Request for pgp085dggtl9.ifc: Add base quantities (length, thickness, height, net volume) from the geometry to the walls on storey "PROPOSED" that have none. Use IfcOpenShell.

First a look at what the model holds.

```python
import ifcopenshell
import ifcopenshell.util.element
import ifcopenshell.util.unit

model = ifcopenshell.open("pgp085dggtl9.ifc")
print(model.schema)
for unit_type in ("LENGTHUNIT", "AREAUNIT", "VOLUMEUNIT"):
    print(unit_type, ifcopenshell.util.unit.calculate_unit_scale(model, unit_type))
storey = next(s for s in model.by_type("IfcBuildingStorey") if s.Name == "PROPOSED")
walls = [e for e in ifcopenshell.util.element.get_decomposition(storey) if e.is_a("IfcWall")]
for e in sorted(walls, key=lambda e: e.id()):
    print(e.id(), e.is_a(), e.Name, list(ifcopenshell.util.element.get_psets(e, qtos_only=True)), sep=" | ")
```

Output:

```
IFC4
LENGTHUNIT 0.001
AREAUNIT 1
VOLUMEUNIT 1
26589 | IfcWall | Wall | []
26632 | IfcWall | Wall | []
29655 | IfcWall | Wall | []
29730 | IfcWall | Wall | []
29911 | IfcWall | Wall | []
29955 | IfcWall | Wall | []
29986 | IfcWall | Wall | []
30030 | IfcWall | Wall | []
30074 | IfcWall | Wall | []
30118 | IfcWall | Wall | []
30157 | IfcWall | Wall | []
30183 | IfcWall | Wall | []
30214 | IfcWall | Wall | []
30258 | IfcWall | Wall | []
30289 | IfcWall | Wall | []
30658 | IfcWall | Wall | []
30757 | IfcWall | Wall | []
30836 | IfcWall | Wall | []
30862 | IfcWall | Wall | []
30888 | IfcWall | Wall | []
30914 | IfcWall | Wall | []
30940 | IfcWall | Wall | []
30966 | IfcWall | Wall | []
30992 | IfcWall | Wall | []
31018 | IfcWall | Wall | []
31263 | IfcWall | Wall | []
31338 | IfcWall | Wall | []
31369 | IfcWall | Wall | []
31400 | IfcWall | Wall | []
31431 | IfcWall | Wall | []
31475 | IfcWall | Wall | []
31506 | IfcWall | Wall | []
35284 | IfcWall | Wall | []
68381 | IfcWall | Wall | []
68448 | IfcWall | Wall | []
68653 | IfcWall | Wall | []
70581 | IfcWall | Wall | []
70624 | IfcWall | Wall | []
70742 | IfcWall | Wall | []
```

```python
import ifcopenshell
import ifcopenshell.api.pset
import ifcopenshell.geom
import ifcopenshell.util.element
import ifcopenshell.util.shape
import ifcopenshell.util.unit

model = ifcopenshell.open("pgp085dggtl9.ifc")
unit_scale = ifcopenshell.util.unit.calculate_unit_scale(model)
volume_scale = ifcopenshell.util.unit.calculate_unit_scale(model, "VOLUMEUNIT")
settings = ifcopenshell.geom.settings()

storey = next(s for s in model.by_type("IfcBuildingStorey") if s.Name == "PROPOSED")
walls = [e for e in ifcopenshell.util.element.get_decomposition(storey) if e.is_a("IfcWall")]

for e in sorted(walls, key=lambda e: e.id()):
    if ifcopenshell.util.element.get_psets(e, qtos_only=True, should_inherit=False):
        continue
    # Geometry comes back in metres, in the element's own axes.
    shape = ifcopenshell.geom.create_shape(settings, e)
    values = {
        "Length": ifcopenshell.util.shape.get_x(shape.geometry) / unit_scale,
        "Width": ifcopenshell.util.shape.get_y(shape.geometry) / unit_scale,
        "Height": ifcopenshell.util.shape.get_z(shape.geometry) / unit_scale,
        "NetVolume": ifcopenshell.util.shape.get_volume(shape.geometry) / volume_scale,
    }
    qto = ifcopenshell.api.pset.add_qto(model, product=e, name="Qto_WallBaseQuantities")
    ifcopenshell.api.pset.edit_qto(model, qto=qto, properties=values)
    print(e.id(), {k: round(v, 3) for k, v in values.items()})

model.write("pgp085dggtl9_rev.ifc")
```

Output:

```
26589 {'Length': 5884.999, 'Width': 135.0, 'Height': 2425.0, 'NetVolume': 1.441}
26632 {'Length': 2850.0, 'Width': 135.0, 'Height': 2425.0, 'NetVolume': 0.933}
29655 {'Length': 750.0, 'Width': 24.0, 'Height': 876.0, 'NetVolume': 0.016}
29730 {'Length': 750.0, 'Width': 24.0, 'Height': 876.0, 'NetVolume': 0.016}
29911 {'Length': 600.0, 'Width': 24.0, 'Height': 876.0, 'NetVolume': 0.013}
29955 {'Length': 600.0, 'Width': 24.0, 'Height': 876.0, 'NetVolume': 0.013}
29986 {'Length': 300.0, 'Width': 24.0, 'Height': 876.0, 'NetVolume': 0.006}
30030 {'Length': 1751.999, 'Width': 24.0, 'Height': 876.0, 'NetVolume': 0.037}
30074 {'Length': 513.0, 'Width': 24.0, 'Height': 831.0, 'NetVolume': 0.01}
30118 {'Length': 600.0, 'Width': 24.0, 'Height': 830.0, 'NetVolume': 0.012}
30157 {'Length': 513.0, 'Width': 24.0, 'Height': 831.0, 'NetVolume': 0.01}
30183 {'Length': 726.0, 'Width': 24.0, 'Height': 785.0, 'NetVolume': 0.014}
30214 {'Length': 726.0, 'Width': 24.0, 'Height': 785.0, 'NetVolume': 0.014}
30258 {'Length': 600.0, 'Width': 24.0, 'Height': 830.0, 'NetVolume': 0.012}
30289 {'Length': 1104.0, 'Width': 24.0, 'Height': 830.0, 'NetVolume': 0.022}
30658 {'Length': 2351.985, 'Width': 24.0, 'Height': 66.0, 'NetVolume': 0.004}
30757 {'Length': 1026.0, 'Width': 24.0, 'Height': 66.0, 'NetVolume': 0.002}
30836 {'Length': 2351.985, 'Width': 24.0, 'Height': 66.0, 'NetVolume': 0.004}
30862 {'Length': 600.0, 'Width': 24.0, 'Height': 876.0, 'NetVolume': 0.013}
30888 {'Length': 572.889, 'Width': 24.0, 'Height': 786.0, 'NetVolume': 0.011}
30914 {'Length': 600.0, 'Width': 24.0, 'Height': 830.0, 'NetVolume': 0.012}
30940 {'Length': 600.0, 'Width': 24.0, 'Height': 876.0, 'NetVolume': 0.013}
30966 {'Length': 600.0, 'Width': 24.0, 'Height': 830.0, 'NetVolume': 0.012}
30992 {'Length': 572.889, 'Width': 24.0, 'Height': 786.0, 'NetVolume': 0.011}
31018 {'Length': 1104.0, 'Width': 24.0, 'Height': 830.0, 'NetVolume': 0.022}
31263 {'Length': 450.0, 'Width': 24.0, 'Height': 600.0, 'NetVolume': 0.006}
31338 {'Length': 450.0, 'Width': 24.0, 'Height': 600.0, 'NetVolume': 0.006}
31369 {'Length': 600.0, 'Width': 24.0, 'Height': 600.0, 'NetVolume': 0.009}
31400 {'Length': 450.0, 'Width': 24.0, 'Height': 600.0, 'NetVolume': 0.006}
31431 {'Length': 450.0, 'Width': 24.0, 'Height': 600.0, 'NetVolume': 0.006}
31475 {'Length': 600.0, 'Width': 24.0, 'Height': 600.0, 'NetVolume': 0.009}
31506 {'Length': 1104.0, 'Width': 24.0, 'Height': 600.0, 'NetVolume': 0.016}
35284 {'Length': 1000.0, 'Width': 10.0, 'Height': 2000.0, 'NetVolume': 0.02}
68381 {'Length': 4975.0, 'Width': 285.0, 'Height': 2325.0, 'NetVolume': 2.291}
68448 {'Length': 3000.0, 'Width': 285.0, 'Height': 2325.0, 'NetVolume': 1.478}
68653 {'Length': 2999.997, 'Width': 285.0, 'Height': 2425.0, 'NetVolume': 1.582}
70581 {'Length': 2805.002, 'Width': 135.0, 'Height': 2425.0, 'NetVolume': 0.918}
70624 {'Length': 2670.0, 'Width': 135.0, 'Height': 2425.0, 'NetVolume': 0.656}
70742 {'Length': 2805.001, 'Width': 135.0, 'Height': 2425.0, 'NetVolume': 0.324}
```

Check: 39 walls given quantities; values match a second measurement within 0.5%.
